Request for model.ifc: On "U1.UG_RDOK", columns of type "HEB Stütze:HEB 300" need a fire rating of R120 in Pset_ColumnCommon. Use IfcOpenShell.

First a look at what the model holds.

```python
import ifcopenshell
import ifcopenshell.util.element

model = ifcopenshell.open("model.ifc")
print(model.schema)
storey = next(s for s in model.by_type("IfcBuildingStorey") if s.Name == "U1.UG_RDOK")
columns = [e for e in ifcopenshell.util.element.get_decomposition(storey) if e.is_a("IfcColumn")]
seen = {}
for e in columns:
    element_type = ifcopenshell.util.element.get_type(e)
    key = (element_type.Name if element_type != e and element_type else None, ifcopenshell.util.element.get_pset(e, "Pset_ColumnCommon", "FireRating"))
    seen[key] = seen.get(key, 0) + 1
for (name, value), count in sorted(seen.items(), key=str):
    print(count, "x", name, "|", value)
```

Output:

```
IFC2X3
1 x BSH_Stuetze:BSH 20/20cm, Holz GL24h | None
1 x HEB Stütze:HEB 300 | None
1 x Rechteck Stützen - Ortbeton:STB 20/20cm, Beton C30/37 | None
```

```python
import ifcopenshell
import ifcopenshell.api.pset
import ifcopenshell.util.element

model = ifcopenshell.open("model.ifc")

storey = next(s for s in model.by_type("IfcBuildingStorey") if s.Name == "U1.UG_RDOK")
columns = [e for e in ifcopenshell.util.element.get_decomposition(storey) if e.is_a("IfcColumn")]

count = 0
for e in columns:
    element_type = ifcopenshell.util.element.get_type(e)
    if element_type in (None, e) or element_type.Name != "HEB Stütze:HEB 300":
        continue
    # add_pset returns the element's existing set when there is one.
    pset = ifcopenshell.api.pset.add_pset(model, product=e, name="Pset_ColumnCommon")
    ifcopenshell.api.pset.edit_pset(model, pset=pset, properties={"FireRating": "R120"})
    count += 1

print(count, "columns updated")

model.write("model_updated.ifc")
```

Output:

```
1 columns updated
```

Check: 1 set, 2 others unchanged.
